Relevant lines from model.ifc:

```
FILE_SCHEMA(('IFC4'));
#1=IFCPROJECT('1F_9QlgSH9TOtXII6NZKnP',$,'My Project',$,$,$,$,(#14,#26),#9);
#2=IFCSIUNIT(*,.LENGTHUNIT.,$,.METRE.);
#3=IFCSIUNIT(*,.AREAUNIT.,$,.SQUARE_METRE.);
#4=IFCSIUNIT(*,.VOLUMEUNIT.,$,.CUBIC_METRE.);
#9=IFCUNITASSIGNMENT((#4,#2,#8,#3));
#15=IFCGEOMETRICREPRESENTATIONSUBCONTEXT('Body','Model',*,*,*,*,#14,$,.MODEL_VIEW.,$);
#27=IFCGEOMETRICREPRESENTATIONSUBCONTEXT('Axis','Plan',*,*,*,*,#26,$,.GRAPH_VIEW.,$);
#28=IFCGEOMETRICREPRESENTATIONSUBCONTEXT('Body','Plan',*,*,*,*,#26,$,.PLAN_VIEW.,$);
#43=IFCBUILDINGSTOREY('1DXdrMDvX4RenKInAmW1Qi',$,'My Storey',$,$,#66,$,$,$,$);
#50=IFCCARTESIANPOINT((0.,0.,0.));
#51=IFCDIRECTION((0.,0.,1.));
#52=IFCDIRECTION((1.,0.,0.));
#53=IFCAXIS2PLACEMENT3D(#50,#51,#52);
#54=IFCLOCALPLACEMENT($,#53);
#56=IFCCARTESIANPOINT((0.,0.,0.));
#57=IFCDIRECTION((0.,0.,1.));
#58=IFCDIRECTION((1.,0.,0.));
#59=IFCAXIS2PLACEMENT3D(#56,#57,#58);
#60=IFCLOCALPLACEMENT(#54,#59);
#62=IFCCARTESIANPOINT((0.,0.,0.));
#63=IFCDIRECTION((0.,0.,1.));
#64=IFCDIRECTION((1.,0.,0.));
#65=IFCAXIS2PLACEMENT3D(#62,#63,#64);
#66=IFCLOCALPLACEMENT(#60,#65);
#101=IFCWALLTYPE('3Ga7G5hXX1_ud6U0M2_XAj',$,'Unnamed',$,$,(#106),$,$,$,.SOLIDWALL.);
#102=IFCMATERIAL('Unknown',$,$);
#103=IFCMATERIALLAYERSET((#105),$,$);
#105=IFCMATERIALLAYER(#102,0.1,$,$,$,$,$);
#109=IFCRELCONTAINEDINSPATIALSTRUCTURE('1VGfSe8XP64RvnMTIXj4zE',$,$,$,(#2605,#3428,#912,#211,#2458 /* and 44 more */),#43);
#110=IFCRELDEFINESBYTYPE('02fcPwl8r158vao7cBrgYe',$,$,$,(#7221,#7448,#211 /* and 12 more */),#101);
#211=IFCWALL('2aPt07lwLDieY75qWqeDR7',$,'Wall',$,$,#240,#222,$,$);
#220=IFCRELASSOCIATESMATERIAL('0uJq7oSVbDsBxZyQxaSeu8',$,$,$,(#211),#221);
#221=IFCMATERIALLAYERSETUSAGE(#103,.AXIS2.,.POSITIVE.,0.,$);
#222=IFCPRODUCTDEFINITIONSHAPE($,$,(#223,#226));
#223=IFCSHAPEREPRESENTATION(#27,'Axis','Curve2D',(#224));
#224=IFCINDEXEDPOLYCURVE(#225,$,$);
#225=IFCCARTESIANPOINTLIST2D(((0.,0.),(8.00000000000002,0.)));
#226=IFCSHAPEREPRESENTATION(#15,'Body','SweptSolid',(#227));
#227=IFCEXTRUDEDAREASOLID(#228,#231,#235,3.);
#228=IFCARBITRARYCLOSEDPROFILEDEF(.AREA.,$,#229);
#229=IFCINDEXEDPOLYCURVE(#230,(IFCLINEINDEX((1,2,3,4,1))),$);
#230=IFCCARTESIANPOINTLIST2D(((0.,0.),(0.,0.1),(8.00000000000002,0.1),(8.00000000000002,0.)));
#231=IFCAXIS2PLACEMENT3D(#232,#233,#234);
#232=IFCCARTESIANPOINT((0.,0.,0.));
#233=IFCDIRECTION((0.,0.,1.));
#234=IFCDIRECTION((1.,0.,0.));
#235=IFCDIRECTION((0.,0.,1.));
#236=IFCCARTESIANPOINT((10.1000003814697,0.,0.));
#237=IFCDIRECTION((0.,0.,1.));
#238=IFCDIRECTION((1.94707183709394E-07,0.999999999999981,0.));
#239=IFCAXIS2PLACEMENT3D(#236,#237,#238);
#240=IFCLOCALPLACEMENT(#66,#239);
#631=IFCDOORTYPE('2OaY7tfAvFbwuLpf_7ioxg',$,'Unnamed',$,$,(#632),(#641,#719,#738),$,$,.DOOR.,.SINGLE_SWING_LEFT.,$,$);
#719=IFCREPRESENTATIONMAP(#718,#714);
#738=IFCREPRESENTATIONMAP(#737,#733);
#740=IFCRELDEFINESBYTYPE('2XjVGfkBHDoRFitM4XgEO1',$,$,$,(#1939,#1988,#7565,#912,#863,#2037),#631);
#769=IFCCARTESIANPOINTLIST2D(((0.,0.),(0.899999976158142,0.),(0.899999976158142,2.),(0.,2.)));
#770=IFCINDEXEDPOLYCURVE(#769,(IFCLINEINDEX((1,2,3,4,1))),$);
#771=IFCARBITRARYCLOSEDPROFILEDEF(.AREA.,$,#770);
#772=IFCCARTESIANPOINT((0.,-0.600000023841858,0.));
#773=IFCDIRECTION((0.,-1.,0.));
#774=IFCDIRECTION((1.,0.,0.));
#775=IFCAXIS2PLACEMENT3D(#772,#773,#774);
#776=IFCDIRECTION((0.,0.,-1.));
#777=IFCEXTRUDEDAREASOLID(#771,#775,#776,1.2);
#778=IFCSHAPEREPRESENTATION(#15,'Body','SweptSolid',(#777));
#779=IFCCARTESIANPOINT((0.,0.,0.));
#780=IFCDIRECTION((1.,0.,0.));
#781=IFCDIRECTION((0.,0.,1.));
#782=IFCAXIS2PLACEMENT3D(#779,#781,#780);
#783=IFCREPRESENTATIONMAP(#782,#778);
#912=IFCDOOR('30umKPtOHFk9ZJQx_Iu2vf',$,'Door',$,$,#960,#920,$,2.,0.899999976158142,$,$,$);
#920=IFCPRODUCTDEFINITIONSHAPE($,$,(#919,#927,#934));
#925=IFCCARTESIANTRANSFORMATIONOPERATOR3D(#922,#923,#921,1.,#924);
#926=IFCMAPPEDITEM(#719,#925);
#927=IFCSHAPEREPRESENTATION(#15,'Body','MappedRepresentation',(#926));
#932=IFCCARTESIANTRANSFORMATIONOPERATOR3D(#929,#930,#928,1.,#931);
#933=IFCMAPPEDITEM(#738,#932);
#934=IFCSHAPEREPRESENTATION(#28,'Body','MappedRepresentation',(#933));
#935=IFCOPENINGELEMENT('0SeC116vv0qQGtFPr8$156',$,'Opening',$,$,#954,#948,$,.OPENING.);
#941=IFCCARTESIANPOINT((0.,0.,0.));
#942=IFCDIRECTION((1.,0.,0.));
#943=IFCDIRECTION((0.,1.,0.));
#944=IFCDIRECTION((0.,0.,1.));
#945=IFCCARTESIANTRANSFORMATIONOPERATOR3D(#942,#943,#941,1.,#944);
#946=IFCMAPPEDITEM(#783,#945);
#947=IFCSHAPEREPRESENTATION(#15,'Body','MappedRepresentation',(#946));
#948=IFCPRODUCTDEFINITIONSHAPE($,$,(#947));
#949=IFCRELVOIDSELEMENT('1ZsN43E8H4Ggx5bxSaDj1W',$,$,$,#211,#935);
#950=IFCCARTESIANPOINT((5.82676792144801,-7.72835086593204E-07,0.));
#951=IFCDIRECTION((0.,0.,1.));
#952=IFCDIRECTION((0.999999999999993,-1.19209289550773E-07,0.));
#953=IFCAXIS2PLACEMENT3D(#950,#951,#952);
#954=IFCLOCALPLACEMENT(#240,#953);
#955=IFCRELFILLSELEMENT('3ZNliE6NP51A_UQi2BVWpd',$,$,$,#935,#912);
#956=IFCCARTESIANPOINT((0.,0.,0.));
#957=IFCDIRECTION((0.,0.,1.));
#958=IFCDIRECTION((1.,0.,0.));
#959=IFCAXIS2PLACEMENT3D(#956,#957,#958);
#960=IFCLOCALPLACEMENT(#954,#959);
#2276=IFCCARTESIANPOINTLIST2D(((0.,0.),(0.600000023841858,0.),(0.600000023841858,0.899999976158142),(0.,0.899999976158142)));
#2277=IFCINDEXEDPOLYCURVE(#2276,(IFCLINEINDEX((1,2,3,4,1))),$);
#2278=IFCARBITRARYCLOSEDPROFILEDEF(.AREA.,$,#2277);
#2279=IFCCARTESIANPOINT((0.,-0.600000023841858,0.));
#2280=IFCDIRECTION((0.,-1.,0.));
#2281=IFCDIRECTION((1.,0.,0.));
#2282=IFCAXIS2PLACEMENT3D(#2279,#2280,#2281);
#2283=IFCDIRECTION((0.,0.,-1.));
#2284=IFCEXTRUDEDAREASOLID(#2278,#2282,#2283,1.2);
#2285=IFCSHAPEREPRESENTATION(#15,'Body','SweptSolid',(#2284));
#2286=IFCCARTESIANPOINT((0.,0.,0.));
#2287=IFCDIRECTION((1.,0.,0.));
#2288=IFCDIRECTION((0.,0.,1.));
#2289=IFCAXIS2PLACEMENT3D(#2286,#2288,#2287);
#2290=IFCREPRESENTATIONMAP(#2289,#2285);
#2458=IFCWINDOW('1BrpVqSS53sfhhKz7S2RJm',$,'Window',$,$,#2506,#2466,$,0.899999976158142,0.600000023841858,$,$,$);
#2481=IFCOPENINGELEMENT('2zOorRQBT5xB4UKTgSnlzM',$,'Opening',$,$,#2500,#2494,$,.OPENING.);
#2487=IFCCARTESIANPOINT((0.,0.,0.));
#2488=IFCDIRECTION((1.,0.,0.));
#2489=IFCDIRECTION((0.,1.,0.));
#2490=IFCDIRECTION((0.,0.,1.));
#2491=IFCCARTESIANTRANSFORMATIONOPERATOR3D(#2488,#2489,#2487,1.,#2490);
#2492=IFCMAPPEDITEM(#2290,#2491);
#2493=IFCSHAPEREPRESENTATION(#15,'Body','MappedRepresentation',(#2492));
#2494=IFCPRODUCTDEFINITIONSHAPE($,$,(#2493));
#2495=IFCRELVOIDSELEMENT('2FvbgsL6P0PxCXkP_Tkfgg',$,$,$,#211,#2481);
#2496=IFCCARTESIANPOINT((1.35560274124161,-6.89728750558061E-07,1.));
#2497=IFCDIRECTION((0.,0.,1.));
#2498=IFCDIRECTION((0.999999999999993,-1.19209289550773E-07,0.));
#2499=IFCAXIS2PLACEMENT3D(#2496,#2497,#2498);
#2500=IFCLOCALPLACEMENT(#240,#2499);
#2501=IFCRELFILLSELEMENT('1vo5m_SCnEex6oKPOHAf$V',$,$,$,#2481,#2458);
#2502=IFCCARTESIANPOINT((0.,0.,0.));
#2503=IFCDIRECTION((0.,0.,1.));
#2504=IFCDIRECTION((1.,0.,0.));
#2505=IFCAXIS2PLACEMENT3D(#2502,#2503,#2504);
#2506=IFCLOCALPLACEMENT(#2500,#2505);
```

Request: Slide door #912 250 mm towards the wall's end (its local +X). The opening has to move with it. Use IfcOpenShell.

```python
import ifcopenshell
import ifcopenshell.api.geometry
import ifcopenshell.util.placement

model = ifcopenshell.open("model.ifc")

door = model.by_guid("30umKPtOHFk9ZJQx_Iu2vf")
opening = door.FillsVoids[0].RelatingOpeningElement
wall = opening.VoidsElements[0].RelatingBuildingElement

wall_matrix = ifcopenshell.util.placement.get_local_placement(wall.ObjectPlacement)
shift = wall_matrix[:3, 0] * 0.25
before = ifcopenshell.util.placement.get_local_placement(door.ObjectPlacement)[:3, 3].copy()

# The door is placed relative to its opening, so it follows when the opening moves.
matrix = ifcopenshell.util.placement.get_local_placement(opening.ObjectPlacement)
matrix[:3, 3] += shift
ifcopenshell.api.geometry.edit_object_placement(
    model, product=opening, matrix=matrix, is_si=False, should_transform_children=True
)

after = ifcopenshell.util.placement.get_local_placement(door.ObjectPlacement)[:3, 3]
print("door moved by", (after - before).round(3) + 0.0)

model.write("model-out.ifc")
```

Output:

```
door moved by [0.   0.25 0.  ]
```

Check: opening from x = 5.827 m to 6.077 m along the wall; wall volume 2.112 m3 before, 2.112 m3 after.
